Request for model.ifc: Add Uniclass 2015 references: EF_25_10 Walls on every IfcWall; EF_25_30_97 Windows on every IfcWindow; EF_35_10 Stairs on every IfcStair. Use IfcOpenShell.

First a look at what the model holds.

```python
import ifcopenshell

model = ifcopenshell.open("model.ifc")
print(model.schema)
print("classifications:", [c.Name for c in model.by_type("IfcClassification")])
for ifc_class in ("IfcDoor", "IfcRoof", "IfcStair", "IfcWall", "IfcWindow"):
    print(ifc_class, len(model.by_type(ifc_class)))
```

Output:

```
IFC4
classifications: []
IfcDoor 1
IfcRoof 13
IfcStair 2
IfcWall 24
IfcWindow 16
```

```python
import ifcopenshell
import ifcopenshell.api.classification

model = ifcopenshell.open("model.ifc")

system = ifcopenshell.api.classification.add_classification(model, classification="Uniclass 2015")

codes = {
    "IfcWall": ("EF_25_10", "Walls"),
    "IfcWindow": ("EF_25_30_97", "Windows"),
    "IfcStair": ("EF_35_10", "Stairs"),
}
for ifc_class, (code, name) in codes.items():
    products = model.by_type(ifc_class)
    ifcopenshell.api.classification.add_reference(
        model, products=products, classification=system, identification=code, name=name
    )
    print(code, len(products))

model.write("model_edited.ifc")
```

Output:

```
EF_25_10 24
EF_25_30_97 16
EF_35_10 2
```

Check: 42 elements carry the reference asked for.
